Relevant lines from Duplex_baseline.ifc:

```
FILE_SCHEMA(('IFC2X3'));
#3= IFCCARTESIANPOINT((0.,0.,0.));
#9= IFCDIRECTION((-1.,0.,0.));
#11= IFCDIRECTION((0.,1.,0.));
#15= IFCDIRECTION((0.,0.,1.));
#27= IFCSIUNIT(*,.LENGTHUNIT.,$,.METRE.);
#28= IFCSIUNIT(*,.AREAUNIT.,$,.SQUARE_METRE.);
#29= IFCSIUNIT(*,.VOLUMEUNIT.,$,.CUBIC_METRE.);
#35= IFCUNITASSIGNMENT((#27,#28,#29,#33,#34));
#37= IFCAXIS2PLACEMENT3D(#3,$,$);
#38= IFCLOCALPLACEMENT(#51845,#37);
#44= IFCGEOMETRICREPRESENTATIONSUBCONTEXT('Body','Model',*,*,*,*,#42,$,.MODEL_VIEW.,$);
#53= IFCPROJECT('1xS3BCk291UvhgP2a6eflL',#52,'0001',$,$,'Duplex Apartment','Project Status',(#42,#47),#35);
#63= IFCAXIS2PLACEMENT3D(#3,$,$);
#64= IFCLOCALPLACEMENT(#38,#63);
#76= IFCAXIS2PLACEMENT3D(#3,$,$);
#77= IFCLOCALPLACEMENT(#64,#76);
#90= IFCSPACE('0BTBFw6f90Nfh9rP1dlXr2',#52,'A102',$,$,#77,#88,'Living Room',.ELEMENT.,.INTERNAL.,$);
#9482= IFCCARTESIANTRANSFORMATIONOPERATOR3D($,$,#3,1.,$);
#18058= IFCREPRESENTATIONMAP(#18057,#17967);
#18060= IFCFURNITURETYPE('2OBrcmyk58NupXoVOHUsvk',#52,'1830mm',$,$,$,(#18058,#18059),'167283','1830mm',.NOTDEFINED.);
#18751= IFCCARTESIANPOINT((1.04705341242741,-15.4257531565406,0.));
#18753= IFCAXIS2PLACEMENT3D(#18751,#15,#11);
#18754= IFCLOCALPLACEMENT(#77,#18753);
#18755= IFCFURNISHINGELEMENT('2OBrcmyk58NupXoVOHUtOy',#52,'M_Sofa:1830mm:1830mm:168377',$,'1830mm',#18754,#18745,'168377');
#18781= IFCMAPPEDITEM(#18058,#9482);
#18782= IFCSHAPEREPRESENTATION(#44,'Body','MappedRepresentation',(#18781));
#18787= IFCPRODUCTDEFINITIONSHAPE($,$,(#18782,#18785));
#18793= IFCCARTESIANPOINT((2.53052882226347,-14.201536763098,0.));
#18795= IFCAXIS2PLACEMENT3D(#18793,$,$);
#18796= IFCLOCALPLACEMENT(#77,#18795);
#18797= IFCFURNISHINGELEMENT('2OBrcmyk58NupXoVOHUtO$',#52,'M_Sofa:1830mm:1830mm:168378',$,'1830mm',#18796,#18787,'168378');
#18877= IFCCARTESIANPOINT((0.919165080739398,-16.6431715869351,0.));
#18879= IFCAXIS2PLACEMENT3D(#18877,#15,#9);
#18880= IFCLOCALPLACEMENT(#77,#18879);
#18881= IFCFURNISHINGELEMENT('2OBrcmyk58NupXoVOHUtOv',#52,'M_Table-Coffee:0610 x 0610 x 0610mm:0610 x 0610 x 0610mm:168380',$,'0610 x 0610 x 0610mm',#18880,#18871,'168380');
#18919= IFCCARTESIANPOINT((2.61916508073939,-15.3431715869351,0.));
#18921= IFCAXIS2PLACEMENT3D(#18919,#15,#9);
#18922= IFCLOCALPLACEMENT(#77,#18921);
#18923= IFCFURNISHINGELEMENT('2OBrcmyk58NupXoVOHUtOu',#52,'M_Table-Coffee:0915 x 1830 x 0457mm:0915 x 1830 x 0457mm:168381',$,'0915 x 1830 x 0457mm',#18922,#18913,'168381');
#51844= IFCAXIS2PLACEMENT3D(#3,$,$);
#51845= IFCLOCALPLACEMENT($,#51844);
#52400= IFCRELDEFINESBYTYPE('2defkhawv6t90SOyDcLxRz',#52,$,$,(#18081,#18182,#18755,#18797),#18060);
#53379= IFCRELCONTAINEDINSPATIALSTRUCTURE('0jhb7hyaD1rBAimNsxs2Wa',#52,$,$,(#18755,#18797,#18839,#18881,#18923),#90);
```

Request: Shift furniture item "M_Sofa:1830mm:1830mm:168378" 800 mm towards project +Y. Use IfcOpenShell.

```python
import ifcopenshell
import ifcopenshell.api.geometry
import ifcopenshell.util.placement
import ifcopenshell.util.unit

model = ifcopenshell.open("Duplex_baseline.ifc")
unit_scale = ifcopenshell.util.unit.calculate_unit_scale(model)

item = model.by_guid("2OBrcmyk58NupXoVOHUtO$")
matrix = ifcopenshell.util.placement.get_local_placement(item.ObjectPlacement)
matrix[1, 3] += 0.8 / unit_scale
ifcopenshell.api.geometry.edit_object_placement(model, product=item, matrix=matrix, is_si=False)

print(ifcopenshell.util.placement.get_local_placement(item.ObjectPlacement).round(3) + 0.0)

model.write("Duplex_baseline_rev.ifc")
```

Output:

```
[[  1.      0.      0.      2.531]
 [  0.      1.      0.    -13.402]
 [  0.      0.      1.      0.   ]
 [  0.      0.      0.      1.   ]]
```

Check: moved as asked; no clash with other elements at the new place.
